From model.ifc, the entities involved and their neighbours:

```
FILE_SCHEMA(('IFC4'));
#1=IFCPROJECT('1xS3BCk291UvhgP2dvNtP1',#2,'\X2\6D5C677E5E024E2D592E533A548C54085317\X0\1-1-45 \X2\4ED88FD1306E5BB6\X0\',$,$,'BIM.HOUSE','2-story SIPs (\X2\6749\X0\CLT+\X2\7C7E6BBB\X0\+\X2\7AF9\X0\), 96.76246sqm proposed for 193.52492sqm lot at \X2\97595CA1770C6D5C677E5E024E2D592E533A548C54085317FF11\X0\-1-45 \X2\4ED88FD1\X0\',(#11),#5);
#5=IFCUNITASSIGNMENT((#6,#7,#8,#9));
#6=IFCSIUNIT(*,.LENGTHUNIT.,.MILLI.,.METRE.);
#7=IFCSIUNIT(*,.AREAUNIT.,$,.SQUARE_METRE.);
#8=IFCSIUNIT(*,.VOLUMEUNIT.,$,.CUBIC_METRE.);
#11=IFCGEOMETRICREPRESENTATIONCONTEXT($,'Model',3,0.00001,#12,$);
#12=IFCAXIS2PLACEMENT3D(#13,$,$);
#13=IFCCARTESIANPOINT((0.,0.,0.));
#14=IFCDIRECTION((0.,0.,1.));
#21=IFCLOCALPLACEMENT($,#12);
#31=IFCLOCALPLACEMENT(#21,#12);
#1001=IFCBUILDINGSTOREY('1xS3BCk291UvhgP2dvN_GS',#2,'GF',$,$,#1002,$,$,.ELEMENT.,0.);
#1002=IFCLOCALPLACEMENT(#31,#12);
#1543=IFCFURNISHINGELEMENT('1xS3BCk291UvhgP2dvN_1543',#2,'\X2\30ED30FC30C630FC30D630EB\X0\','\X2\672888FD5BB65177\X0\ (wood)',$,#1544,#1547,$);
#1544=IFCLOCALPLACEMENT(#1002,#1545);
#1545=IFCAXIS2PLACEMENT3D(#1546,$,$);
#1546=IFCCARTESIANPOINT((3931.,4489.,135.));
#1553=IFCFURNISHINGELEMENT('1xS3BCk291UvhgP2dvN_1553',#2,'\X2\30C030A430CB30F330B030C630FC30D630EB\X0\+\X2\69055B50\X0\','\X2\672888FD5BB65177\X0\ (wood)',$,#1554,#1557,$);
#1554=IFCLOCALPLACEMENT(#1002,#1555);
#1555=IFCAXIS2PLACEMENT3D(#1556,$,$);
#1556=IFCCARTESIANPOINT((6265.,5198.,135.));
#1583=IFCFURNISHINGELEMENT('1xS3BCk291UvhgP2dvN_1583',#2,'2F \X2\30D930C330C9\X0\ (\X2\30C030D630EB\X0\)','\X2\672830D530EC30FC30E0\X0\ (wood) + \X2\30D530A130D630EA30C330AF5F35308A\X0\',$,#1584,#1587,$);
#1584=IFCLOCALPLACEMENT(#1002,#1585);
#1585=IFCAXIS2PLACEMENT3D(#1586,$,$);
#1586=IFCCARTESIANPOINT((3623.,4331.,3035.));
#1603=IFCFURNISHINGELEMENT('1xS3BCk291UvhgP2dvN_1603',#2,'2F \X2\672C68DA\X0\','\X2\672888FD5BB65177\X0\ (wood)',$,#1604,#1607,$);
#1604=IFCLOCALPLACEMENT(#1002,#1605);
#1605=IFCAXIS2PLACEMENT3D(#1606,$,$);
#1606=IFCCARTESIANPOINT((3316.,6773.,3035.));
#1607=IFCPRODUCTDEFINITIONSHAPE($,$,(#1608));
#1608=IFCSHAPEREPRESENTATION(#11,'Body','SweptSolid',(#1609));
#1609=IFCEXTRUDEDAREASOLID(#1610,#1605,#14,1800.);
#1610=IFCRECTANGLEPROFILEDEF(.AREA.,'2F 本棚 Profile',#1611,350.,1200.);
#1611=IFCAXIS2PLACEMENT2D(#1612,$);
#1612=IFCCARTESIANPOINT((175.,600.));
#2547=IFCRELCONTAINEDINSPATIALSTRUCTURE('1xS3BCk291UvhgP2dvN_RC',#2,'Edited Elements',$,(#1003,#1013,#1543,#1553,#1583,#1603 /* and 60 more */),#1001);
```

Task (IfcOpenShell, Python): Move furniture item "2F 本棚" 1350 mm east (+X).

```python
import ifcopenshell
import ifcopenshell.api.geometry
import ifcopenshell.util.placement
import ifcopenshell.util.unit

model = ifcopenshell.open("model.ifc")
unit_scale = ifcopenshell.util.unit.calculate_unit_scale(model)

item = model.by_guid("1xS3BCk291UvhgP2dvN_1603")
matrix = ifcopenshell.util.placement.get_local_placement(item.ObjectPlacement)
matrix[0, 3] += 1.35 / unit_scale
ifcopenshell.api.geometry.edit_object_placement(model, product=item, matrix=matrix, is_si=False)

print(ifcopenshell.util.placement.get_local_placement(item.ObjectPlacement).round(3) + 0.0)

model.write("model_v2.ifc")
```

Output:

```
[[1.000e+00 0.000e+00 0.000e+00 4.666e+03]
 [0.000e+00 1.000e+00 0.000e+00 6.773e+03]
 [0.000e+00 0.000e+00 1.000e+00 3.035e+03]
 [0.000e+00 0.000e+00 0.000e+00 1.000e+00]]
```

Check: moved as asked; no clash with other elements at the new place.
